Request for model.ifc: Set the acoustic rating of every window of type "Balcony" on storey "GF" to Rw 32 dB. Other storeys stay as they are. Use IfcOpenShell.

First a look at what the model holds.

```python
import ifcopenshell
import ifcopenshell.util.element

model = ifcopenshell.open("model.ifc")
print(model.schema)
storey = next(s for s in model.by_type("IfcBuildingStorey") if s.Name == "GF")
windows = [e for e in ifcopenshell.util.element.get_decomposition(storey) if e.is_a("IfcWindow")]
seen = {}
for e in windows:
    element_type = ifcopenshell.util.element.get_type(e)
    key = (element_type.Name if element_type != e and element_type else None, ifcopenshell.util.element.get_pset(e, "Pset_WindowCommon", "AcousticRating"))
    seen[key] = seen.get(key, 0) + 1
for (name, value), count in sorted(seen.items(), key=str):
    print(count, "x", name, "|", value)
```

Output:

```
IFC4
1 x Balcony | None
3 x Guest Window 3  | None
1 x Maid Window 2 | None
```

```python
import ifcopenshell
import ifcopenshell.api.pset
import ifcopenshell.util.element

model = ifcopenshell.open("model.ifc")

storey = next(s for s in model.by_type("IfcBuildingStorey") if s.Name == "GF")
windows = [e for e in ifcopenshell.util.element.get_decomposition(storey) if e.is_a("IfcWindow")]

count = 0
for e in windows:
    element_type = ifcopenshell.util.element.get_type(e)
    if element_type in (None, e) or element_type.Name != "Balcony":
        continue
    # add_pset returns the element's existing set when there is one.
    pset = ifcopenshell.api.pset.add_pset(model, product=e, name="Pset_WindowCommon")
    ifcopenshell.api.pset.edit_pset(model, pset=pset, properties={"AcousticRating": "Rw 32 dB"})
    count += 1

print(count, "windows updated")

model.write("model_v2.ifc")
```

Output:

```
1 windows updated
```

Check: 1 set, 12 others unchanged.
